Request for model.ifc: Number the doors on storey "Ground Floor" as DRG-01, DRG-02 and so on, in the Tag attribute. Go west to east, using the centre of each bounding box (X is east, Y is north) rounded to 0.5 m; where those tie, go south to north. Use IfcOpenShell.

First a look at what the model holds.

```python
import ifcopenshell
import ifcopenshell.util.element
import ifcopenshell.util.placement

model = ifcopenshell.open("model.ifc")
print(model.schema)
storey = next(s for s in model.by_type("IfcBuildingStorey") if s.Name == "Ground Floor")
doors = [e for e in ifcopenshell.util.element.get_decomposition(storey) if e.is_a("IfcDoor")]
for e in sorted(doors, key=lambda e: e.id()):
    origin = ifcopenshell.util.placement.get_local_placement(e.ObjectPlacement)[:3, 3]
    print(e.id(), e.Tag, e.Name, origin.round(2) + 0.0, sep=" | ")
```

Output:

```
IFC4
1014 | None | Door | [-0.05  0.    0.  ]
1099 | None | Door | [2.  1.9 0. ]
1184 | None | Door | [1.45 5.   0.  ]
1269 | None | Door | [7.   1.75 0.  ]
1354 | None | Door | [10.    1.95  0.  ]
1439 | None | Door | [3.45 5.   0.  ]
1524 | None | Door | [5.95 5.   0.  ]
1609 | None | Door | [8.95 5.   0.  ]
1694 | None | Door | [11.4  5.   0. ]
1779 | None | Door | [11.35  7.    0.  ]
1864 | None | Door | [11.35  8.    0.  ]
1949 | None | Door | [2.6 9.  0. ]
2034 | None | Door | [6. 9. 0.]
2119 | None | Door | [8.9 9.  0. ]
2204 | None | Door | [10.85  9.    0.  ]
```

```python
import ifcopenshell
import ifcopenshell.geom
import ifcopenshell.util.element
import ifcopenshell.util.shape

model = ifcopenshell.open("model.ifc")
settings = ifcopenshell.geom.settings()
settings.set("use-world-coords", True)


def centre(element):
    shape = ifcopenshell.geom.create_shape(settings, element)
    return ifcopenshell.util.shape.get_bbox_centroid(shape.geometry)


storey = next(s for s in model.by_type("IfcBuildingStorey") if s.Name == "Ground Floor")
doors = [e for e in ifcopenshell.util.element.get_decomposition(storey) if e.is_a("IfcDoor")]

# Insertion points can sit at a corner or the storey origin, so sort by the geometry (in metres).
centres = {e: centre(e) for e in doors}
doors.sort(key=lambda e: (round(centres[e][0] / 0.5), centres[e][1]))

for i, e in enumerate(doors, start=1):
    number = f"DRG-{i:02d}"
    e.Tag = number
    print(e.id(), number)

model.write("model-out.ifc")
```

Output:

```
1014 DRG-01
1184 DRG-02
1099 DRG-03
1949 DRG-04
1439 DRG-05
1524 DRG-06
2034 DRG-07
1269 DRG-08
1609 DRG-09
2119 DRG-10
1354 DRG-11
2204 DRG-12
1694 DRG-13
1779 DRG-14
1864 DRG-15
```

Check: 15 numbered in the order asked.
